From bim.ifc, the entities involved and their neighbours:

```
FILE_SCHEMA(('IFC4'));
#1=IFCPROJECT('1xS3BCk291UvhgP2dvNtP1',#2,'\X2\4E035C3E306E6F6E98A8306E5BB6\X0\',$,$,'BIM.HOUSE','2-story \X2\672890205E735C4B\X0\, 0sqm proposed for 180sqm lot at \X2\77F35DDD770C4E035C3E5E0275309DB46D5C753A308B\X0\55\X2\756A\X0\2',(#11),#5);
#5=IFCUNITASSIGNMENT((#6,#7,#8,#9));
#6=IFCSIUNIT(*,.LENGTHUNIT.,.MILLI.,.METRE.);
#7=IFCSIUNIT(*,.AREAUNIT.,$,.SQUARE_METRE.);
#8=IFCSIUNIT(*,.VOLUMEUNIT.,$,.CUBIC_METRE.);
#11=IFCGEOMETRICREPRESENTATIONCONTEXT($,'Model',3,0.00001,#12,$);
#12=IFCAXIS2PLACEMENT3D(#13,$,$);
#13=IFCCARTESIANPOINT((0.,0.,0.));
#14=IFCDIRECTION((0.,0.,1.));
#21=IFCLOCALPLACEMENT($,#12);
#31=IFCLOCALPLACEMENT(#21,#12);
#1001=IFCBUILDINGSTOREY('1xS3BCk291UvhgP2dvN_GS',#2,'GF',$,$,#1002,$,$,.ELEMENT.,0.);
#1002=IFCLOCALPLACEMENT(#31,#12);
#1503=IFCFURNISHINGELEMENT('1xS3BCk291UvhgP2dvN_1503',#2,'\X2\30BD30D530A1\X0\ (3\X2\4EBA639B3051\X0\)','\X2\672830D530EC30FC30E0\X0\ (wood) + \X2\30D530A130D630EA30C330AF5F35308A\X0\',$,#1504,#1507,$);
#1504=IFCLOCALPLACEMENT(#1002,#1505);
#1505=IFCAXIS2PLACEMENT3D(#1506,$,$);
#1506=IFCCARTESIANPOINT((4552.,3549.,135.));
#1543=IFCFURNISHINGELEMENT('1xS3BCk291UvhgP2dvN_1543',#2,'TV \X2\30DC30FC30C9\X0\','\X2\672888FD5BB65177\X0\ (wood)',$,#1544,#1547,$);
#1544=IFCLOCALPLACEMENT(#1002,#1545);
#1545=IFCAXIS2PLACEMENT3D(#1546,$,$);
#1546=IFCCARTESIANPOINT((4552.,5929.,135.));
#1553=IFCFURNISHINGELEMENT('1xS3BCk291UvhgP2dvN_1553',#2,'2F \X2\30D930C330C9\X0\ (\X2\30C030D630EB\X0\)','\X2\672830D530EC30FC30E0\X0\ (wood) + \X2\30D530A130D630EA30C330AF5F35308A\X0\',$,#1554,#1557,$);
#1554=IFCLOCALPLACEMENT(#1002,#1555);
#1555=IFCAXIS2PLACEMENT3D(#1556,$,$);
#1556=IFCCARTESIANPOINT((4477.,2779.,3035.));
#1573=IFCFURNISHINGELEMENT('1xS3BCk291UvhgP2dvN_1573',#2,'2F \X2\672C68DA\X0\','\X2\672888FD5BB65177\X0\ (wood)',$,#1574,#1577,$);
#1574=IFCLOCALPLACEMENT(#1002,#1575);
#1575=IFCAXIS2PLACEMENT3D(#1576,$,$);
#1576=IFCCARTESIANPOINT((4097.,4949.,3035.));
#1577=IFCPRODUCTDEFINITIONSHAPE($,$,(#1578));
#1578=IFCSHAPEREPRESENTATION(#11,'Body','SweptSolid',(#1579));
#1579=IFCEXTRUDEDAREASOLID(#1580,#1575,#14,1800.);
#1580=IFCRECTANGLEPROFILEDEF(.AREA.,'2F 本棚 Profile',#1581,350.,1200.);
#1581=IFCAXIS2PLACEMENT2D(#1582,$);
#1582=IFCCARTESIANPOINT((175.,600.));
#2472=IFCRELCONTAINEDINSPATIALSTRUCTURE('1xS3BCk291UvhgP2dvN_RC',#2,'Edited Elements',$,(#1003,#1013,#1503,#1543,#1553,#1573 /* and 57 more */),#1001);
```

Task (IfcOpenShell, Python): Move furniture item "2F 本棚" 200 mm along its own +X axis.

```python
import ifcopenshell
import ifcopenshell.api.geometry
import ifcopenshell.util.placement
import ifcopenshell.util.unit

model = ifcopenshell.open("bim.ifc")
unit_scale = ifcopenshell.util.unit.calculate_unit_scale(model)

item = model.by_guid("1xS3BCk291UvhgP2dvN_1573")
matrix = ifcopenshell.util.placement.get_local_placement(item.ObjectPlacement)
matrix[:3, 3] += matrix[:3, 0] * 0.2 / unit_scale
ifcopenshell.api.geometry.edit_object_placement(model, product=item, matrix=matrix, is_si=False)

print(ifcopenshell.util.placement.get_local_placement(item.ObjectPlacement).round(3) + 0.0)

model.write("bim_edited.ifc")
```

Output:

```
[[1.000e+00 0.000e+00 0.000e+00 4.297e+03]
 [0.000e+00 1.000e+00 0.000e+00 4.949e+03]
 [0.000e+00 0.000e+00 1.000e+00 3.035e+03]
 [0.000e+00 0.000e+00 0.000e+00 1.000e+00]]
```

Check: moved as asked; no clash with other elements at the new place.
